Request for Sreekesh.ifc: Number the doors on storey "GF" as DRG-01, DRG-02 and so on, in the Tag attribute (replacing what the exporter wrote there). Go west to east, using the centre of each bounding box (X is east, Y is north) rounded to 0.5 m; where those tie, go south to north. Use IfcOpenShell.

First a look at what the model holds.

```python
import ifcopenshell
import ifcopenshell.util.element
import ifcopenshell.util.placement

model = ifcopenshell.open("Sreekesh.ifc")
print(model.schema)
storey = next(s for s in model.by_type("IfcBuildingStorey") if s.Name == "GF")
doors = [e for e in ifcopenshell.util.element.get_decomposition(storey) if e.is_a("IfcDoor")]
for e in sorted(doors, key=lambda e: e.id()):
    origin = ifcopenshell.util.placement.get_local_placement(e.ObjectPlacement)[:3, 3]
    print(e.id(), e.Tag, e.Name, origin.round(2) + 0.0, sep=" | ")
```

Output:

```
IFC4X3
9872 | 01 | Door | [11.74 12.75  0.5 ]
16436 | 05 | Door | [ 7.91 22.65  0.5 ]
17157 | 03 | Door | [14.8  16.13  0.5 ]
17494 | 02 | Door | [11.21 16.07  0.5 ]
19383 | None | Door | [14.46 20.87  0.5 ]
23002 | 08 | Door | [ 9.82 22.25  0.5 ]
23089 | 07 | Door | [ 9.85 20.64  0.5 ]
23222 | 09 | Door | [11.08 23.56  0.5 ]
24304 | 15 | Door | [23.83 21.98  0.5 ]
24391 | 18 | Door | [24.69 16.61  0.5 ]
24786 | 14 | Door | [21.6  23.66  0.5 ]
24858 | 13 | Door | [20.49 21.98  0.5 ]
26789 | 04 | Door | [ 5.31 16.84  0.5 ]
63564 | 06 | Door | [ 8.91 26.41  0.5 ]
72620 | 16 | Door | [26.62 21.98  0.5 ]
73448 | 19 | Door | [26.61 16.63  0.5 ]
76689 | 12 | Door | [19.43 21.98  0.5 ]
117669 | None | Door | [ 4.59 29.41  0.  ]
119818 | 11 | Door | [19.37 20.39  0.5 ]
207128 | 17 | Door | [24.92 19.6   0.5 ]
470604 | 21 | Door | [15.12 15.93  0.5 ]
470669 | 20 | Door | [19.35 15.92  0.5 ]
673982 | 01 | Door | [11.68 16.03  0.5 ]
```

```python
import ifcopenshell
import ifcopenshell.geom
import ifcopenshell.util.element
import ifcopenshell.util.shape

model = ifcopenshell.open("Sreekesh.ifc")
settings = ifcopenshell.geom.settings()
settings.set("use-world-coords", True)


def centre(element):
    shape = ifcopenshell.geom.create_shape(settings, element)
    return ifcopenshell.util.shape.get_bbox_centroid(shape.geometry)


storey = next(s for s in model.by_type("IfcBuildingStorey") if s.Name == "GF")
doors = [e for e in ifcopenshell.util.element.get_decomposition(storey) if e.is_a("IfcDoor")]

# Insertion points can sit at a corner or the storey origin, so sort by the geometry (in metres).
centres = {e: centre(e) for e in doors}
doors.sort(key=lambda e: (round(centres[e][0] / 0.5), centres[e][1]))

for i, e in enumerate(doors, start=1):
    number = f"DRG-{i:02d}"
    e.Tag = number
    print(e.id(), number)

model.write("Sreekesh_v2.ifc")
```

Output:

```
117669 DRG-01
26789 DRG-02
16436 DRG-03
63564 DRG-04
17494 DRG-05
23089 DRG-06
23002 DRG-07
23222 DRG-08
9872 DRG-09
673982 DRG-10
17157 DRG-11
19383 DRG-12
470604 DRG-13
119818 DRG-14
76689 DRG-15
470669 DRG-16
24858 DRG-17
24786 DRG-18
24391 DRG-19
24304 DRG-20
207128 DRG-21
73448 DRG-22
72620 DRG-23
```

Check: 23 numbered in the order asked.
